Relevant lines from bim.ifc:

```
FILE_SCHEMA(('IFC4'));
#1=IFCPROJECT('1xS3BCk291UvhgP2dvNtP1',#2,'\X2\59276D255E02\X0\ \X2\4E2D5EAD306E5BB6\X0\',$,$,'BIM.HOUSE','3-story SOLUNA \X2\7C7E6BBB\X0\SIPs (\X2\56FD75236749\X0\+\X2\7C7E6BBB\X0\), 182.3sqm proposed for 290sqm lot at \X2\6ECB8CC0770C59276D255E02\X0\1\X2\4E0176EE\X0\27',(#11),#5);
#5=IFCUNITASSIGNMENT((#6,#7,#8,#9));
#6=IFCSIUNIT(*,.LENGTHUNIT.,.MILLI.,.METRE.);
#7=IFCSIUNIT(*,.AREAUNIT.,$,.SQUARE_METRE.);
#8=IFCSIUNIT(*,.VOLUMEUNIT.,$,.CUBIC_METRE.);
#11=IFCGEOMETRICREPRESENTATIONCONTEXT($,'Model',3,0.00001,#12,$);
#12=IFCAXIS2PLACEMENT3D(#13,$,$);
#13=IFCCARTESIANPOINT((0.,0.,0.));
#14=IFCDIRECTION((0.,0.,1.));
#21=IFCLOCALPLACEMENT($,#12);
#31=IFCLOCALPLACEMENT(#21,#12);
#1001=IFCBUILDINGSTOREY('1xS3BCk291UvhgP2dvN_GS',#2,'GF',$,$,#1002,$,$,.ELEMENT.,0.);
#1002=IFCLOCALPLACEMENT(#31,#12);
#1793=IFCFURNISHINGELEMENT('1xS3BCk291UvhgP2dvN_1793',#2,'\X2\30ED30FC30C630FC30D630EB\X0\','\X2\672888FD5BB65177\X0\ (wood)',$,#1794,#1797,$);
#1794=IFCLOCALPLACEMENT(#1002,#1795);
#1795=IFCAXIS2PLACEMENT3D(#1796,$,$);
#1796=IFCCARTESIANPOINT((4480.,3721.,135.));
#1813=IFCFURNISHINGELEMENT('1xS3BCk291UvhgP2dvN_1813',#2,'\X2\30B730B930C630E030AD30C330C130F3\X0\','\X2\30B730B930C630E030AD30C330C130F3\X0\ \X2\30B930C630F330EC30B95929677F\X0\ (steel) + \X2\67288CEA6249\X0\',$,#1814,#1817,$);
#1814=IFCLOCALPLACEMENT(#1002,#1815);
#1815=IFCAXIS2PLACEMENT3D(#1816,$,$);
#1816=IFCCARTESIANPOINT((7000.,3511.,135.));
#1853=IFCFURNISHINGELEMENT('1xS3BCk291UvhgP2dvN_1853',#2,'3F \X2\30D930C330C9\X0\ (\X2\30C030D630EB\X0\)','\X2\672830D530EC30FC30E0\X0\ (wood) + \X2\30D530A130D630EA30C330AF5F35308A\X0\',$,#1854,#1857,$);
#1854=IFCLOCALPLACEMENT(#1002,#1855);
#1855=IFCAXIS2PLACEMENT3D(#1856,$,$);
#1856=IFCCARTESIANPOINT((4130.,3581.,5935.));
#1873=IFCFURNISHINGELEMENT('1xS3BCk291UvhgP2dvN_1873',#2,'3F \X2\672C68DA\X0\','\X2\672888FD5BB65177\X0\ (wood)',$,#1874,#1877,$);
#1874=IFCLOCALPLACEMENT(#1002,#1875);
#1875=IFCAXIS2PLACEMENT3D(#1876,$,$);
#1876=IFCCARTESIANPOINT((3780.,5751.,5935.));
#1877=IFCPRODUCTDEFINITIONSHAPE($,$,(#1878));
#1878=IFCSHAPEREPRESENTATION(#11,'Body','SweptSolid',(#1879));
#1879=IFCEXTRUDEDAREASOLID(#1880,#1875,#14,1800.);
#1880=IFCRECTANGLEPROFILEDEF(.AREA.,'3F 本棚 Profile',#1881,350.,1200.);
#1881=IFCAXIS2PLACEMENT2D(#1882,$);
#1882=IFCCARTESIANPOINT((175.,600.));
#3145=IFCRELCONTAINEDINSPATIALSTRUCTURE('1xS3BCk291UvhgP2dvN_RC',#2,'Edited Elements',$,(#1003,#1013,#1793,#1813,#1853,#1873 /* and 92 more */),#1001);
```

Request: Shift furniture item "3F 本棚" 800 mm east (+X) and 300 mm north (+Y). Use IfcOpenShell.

```python
import ifcopenshell
import ifcopenshell.api.geometry
import ifcopenshell.util.placement
import ifcopenshell.util.unit

model = ifcopenshell.open("bim.ifc")
unit_scale = ifcopenshell.util.unit.calculate_unit_scale(model)

item = model.by_guid("1xS3BCk291UvhgP2dvN_1873")
matrix = ifcopenshell.util.placement.get_local_placement(item.ObjectPlacement)
matrix[0, 3] += 0.8 / unit_scale
matrix[1, 3] += 0.3 / unit_scale
ifcopenshell.api.geometry.edit_object_placement(model, product=item, matrix=matrix, is_si=False)

print(ifcopenshell.util.placement.get_local_placement(item.ObjectPlacement).round(3) + 0.0)

model.write("bim_edited.ifc")
```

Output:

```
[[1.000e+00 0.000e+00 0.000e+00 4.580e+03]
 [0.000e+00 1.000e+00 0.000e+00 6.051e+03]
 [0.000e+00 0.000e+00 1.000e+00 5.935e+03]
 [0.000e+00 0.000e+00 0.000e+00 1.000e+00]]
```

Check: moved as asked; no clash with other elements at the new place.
